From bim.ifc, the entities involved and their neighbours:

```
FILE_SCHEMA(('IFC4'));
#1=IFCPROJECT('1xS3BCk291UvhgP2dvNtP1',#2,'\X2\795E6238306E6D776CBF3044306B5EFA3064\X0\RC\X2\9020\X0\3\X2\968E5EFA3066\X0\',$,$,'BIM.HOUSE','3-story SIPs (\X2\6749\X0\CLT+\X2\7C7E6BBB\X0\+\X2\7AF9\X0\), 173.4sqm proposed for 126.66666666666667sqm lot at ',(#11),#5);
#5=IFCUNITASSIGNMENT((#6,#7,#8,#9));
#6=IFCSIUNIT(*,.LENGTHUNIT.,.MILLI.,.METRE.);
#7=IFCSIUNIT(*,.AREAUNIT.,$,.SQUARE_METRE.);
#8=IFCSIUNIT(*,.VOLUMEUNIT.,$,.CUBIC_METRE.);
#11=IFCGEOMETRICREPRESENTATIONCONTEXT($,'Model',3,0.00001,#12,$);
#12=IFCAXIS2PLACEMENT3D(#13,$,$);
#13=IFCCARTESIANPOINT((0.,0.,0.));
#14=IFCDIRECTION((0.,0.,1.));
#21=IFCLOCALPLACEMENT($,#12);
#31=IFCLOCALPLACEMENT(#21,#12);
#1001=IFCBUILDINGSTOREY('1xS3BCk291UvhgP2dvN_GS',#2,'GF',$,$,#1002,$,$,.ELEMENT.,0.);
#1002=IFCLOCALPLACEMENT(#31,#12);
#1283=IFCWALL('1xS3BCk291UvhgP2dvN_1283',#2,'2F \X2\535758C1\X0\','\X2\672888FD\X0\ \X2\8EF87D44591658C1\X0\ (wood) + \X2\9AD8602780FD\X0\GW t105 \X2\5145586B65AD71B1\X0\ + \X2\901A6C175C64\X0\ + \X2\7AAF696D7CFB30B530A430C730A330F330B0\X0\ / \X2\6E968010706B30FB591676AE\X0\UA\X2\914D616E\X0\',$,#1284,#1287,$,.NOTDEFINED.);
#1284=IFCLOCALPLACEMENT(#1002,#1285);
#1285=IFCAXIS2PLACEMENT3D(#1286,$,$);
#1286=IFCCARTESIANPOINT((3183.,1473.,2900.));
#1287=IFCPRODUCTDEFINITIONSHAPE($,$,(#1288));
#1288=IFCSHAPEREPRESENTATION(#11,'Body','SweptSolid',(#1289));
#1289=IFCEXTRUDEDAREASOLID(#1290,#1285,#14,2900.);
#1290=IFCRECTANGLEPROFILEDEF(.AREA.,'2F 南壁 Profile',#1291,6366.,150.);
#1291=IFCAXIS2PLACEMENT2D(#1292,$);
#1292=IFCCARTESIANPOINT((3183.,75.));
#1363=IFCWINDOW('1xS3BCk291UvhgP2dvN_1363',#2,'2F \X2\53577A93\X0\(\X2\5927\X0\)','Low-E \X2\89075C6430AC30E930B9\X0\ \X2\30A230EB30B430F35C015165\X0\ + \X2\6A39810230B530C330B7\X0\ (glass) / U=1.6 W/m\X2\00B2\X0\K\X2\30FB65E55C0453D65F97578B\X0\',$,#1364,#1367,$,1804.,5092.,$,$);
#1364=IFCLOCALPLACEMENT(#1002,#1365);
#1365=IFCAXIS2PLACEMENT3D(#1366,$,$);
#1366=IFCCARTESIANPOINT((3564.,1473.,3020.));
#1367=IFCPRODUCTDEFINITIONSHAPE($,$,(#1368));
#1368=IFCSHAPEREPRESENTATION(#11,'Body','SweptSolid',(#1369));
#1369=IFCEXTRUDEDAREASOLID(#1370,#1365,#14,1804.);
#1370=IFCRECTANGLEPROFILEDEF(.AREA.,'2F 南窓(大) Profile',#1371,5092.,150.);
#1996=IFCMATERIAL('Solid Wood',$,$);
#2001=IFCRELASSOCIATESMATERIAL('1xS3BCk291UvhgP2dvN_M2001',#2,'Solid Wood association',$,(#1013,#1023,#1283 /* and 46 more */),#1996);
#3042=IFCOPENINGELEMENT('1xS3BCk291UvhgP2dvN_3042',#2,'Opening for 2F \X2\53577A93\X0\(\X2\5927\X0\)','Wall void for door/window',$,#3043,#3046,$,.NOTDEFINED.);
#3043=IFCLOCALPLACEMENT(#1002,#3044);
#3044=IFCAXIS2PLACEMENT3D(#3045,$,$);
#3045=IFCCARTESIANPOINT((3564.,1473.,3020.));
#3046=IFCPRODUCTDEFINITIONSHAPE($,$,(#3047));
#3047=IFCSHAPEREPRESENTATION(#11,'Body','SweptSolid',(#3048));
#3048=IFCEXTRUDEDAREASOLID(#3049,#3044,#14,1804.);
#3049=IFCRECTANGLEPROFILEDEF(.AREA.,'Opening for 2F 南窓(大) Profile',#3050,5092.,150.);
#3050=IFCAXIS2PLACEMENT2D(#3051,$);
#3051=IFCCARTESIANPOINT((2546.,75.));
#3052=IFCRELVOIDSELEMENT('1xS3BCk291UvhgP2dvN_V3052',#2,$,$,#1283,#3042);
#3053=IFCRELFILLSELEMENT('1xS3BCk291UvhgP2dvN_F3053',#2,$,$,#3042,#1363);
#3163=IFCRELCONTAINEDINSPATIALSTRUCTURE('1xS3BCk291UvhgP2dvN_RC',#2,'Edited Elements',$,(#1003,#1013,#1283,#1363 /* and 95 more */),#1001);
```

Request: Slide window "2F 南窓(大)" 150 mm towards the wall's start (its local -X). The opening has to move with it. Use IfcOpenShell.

```python
import ifcopenshell
import ifcopenshell.api.geometry
import ifcopenshell.util.placement

model = ifcopenshell.open("bim.ifc")

window = model.by_guid("1xS3BCk291UvhgP2dvN_1363")
opening = window.FillsVoids[0].RelatingOpeningElement
wall = opening.VoidsElements[0].RelatingBuildingElement

wall_matrix = ifcopenshell.util.placement.get_local_placement(wall.ObjectPlacement)
shift = wall_matrix[:3, 0] * -150.0
before = ifcopenshell.util.placement.get_local_placement(window.ObjectPlacement)[:3, 3].copy()

# The window is not placed relative to its opening, so move both.
for product in (opening, window):
    matrix = ifcopenshell.util.placement.get_local_placement(product.ObjectPlacement)
    matrix[:3, 3] += shift
    ifcopenshell.api.geometry.edit_object_placement(model, product=product, matrix=matrix, is_si=False)

after = ifcopenshell.util.placement.get_local_placement(window.ObjectPlacement)[:3, 3]
print("window moved by", (after - before).round(3) + 0.0)

model.write("bim_edited.ifc")
```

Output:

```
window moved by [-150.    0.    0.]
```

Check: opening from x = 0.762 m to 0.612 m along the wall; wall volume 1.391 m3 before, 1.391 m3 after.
